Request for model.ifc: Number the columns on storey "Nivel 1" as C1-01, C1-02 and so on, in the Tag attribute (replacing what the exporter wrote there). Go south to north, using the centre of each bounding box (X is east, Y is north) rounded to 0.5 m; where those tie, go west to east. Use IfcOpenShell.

First a look at what the model holds.

```python
import ifcopenshell
import ifcopenshell.util.element
import ifcopenshell.util.placement

model = ifcopenshell.open("model.ifc")
print(model.schema)
storey = next(s for s in model.by_type("IfcBuildingStorey") if s.Name == "Nivel 1")
columns = [e for e in ifcopenshell.util.element.get_decomposition(storey) if e.is_a("IfcColumn")]
for e in sorted(columns, key=lambda e: e.id()):
    origin = ifcopenshell.util.placement.get_local_placement(e.ObjectPlacement)[:3, 3]
    print(e.id(), e.Tag, e.Name, origin.round(2) + 0.0, sep=" | ")
```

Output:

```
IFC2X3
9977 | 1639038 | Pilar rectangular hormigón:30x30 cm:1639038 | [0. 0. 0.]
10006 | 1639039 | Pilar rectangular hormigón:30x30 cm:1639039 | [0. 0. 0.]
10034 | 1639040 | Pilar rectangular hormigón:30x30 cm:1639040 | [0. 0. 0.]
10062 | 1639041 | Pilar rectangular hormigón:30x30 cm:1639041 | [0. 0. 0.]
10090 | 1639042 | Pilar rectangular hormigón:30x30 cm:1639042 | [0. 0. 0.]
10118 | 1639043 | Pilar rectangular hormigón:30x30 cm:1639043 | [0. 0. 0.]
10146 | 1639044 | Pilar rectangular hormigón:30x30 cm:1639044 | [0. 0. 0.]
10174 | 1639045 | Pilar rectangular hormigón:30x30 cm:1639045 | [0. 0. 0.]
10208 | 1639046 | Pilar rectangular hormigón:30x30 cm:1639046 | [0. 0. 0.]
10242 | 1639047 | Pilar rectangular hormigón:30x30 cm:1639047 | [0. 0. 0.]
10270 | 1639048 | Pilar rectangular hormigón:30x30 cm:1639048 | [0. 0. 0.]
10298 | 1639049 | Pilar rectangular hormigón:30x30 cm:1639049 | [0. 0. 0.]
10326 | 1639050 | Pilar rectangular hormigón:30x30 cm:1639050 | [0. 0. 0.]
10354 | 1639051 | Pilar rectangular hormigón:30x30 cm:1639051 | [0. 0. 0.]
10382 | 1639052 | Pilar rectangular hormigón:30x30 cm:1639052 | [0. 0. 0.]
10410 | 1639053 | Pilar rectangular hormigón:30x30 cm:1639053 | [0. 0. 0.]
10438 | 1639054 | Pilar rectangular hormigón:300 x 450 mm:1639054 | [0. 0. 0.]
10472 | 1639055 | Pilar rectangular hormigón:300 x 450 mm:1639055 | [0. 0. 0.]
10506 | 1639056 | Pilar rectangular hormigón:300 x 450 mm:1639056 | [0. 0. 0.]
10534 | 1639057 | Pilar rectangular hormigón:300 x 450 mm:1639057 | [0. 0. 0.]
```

```python
import ifcopenshell
import ifcopenshell.geom
import ifcopenshell.util.element
import ifcopenshell.util.shape

model = ifcopenshell.open("model.ifc")
settings = ifcopenshell.geom.settings()
settings.set("use-world-coords", True)


def centre(element):
    shape = ifcopenshell.geom.create_shape(settings, element)
    return ifcopenshell.util.shape.get_bbox_centroid(shape.geometry)


storey = next(s for s in model.by_type("IfcBuildingStorey") if s.Name == "Nivel 1")
columns = [e for e in ifcopenshell.util.element.get_decomposition(storey) if e.is_a("IfcColumn")]

# Insertion points can sit at a corner or the storey origin, so sort by the geometry (in metres).
centres = {e: centre(e) for e in columns}
columns.sort(key=lambda e: (round(centres[e][1] / 0.5), centres[e][0]))

for i, e in enumerate(columns, start=1):
    number = f"C1-{i:02d}"
    e.Tag = number
    print(e.id(), number)

model.write("model_v2.ifc")
```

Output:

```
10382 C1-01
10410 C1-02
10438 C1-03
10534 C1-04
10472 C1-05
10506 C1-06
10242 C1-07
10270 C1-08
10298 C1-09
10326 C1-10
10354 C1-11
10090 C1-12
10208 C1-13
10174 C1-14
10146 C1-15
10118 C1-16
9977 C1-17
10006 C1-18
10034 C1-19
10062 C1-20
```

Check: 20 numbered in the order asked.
